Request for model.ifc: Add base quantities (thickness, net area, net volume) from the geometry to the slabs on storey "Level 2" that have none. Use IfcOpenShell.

First a look at what the model holds.

```python
import ifcopenshell
import ifcopenshell.util.element
import ifcopenshell.util.unit

model = ifcopenshell.open("model.ifc")
print(model.schema)
for unit_type in ("LENGTHUNIT", "AREAUNIT", "VOLUMEUNIT"):
    print(unit_type, ifcopenshell.util.unit.calculate_unit_scale(model, unit_type))
storey = next(s for s in model.by_type("IfcBuildingStorey") if s.Name == "Level 2")
slabs = [e for e in ifcopenshell.util.element.get_decomposition(storey) if e.is_a("IfcSlab")]
for e in sorted(slabs, key=lambda e: e.id()):
    print(e.id(), e.is_a(), e.Name, list(ifcopenshell.util.element.get_psets(e, qtos_only=True)), sep=" | ")
```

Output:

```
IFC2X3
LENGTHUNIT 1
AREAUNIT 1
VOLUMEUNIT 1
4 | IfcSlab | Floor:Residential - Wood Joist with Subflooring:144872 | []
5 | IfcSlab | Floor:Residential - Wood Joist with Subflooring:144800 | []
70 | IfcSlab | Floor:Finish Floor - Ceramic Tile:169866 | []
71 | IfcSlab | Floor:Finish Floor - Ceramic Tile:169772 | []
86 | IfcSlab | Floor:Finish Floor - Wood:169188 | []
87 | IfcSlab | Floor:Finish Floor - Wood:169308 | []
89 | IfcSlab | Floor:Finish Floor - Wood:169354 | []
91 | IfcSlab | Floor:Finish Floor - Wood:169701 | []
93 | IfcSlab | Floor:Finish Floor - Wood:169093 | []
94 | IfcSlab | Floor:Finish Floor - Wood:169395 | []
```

```python
import ifcopenshell
import ifcopenshell.api.pset
import ifcopenshell.geom
import ifcopenshell.util.element
import ifcopenshell.util.shape
import ifcopenshell.util.unit

model = ifcopenshell.open("model.ifc")
unit_scale = ifcopenshell.util.unit.calculate_unit_scale(model)
area_scale = ifcopenshell.util.unit.calculate_unit_scale(model, "AREAUNIT")
volume_scale = ifcopenshell.util.unit.calculate_unit_scale(model, "VOLUMEUNIT")
settings = ifcopenshell.geom.settings()

storey = next(s for s in model.by_type("IfcBuildingStorey") if s.Name == "Level 2")
slabs = [e for e in ifcopenshell.util.element.get_decomposition(storey) if e.is_a("IfcSlab")]

for e in sorted(slabs, key=lambda e: e.id()):
    if ifcopenshell.util.element.get_psets(e, qtos_only=True, should_inherit=False):
        continue
    # Geometry comes back in metres, in the element's own axes.
    shape = ifcopenshell.geom.create_shape(settings, e)
    values = {
        "Width": ifcopenshell.util.shape.get_z(shape.geometry) / unit_scale,
        "NetArea": ifcopenshell.util.shape.get_footprint_area(shape.geometry) / area_scale,
        "NetVolume": ifcopenshell.util.shape.get_volume(shape.geometry) / volume_scale,
    }
    qto = ifcopenshell.api.pset.add_qto(model, product=e, name="BaseQuantities")
    ifcopenshell.api.pset.edit_qto(model, qto=qto, properties=values)
    print(e.id(), {k: round(v, 3) for k, v in values.items()})

model.write("model_updated.ifc")
```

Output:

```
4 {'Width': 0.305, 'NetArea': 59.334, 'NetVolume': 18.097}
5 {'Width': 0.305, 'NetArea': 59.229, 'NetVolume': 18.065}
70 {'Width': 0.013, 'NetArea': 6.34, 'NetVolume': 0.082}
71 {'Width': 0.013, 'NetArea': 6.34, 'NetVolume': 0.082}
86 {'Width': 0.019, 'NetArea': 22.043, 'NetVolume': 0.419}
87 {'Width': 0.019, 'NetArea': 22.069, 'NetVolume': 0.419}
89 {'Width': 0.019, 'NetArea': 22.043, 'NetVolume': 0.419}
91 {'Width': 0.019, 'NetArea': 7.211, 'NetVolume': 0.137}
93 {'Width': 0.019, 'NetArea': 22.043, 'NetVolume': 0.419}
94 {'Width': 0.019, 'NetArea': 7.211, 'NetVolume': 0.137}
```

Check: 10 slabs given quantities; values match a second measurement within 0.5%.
